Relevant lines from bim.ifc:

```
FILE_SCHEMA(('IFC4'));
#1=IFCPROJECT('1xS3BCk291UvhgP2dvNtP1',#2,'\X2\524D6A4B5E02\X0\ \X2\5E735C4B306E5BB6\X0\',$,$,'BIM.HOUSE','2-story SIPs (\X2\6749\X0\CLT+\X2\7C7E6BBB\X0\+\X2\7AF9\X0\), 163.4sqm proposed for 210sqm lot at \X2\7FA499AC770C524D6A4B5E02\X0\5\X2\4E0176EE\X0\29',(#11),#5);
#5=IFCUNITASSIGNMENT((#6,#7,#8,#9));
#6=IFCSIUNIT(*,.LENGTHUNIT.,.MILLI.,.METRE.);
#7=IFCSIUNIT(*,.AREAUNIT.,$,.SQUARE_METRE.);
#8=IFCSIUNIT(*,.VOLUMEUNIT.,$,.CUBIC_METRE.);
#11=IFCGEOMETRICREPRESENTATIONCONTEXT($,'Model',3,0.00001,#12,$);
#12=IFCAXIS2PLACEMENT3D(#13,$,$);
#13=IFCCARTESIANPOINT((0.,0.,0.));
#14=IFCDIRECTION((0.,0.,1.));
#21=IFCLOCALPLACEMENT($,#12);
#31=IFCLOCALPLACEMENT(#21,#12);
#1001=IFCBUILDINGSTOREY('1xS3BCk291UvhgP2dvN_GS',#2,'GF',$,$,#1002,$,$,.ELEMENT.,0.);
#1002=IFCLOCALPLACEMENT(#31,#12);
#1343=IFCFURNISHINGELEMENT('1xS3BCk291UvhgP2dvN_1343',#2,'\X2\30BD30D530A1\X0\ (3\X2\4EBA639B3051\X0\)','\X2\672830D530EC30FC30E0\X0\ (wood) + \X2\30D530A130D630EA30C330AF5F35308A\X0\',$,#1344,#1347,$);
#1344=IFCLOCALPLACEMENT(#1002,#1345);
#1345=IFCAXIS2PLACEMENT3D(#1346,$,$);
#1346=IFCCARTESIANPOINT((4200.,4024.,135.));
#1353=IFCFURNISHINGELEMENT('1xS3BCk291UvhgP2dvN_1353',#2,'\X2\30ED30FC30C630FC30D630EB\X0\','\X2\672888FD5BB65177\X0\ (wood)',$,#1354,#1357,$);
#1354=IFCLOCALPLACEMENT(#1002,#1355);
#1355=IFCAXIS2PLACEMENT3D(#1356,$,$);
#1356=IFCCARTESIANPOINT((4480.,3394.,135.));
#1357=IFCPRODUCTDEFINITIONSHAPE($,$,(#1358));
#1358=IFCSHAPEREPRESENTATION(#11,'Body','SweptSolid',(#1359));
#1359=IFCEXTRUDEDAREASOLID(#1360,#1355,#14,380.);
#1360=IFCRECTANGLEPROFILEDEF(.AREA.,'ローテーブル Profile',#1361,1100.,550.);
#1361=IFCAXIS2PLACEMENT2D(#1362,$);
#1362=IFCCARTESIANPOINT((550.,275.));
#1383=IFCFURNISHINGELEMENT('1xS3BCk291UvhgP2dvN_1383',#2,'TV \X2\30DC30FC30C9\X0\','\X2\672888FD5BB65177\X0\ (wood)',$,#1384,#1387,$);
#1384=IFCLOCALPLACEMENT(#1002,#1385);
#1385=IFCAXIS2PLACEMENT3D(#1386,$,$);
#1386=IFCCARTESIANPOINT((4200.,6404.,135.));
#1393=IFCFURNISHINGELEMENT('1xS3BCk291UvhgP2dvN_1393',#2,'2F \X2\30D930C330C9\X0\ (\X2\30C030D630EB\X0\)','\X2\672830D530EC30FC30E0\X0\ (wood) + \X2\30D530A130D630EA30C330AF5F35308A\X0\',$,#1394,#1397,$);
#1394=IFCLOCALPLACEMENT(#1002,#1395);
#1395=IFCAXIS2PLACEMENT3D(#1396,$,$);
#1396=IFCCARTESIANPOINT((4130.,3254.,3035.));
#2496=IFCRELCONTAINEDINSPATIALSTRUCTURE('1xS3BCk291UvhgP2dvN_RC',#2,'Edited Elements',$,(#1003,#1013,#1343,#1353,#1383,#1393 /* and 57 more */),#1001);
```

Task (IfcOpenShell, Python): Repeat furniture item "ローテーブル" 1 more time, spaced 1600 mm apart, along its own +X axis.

```python
import ifcopenshell
import ifcopenshell.api.geometry
import ifcopenshell.api.root
import ifcopenshell.util.element
import ifcopenshell.util.placement

model = ifcopenshell.open("bim.ifc")


def reuse_history(source, copy):
    """copy_class also copies each property set's owner history, people and application; keep the originals."""
    for rel in copy.IsDefinedBy:
        if rel.is_a("IfcRelDefinesByProperties") and (history := rel.RelatingPropertyDefinition.OwnerHistory):
            rel.RelatingPropertyDefinition.OwnerHistory = source.OwnerHistory
            ifcopenshell.util.element.remove_deep2(model, history)


source = model.by_guid("1xS3BCk291UvhgP2dvN_1353")
base = ifcopenshell.util.placement.get_local_placement(source.ObjectPlacement)
step = base[:3, 0] * 1600.0

for i in range(1, 2):
    copy = ifcopenshell.api.root.copy_class(model, product=source)
    copy.Representation = ifcopenshell.util.element.copy_deep(
        model, source.Representation, exclude=["IfcGeometricRepresentationContext", "IfcRepresentationMap"]
    )
    reuse_history(source, copy)
    matrix = base.copy()
    matrix[:3, 3] += i * step
    print("added at", matrix[:3, 3].round(3) + 0.0)
    ifcopenshell.api.geometry.edit_object_placement(model, product=copy, matrix=matrix, is_si=False)

model.write("bim-out.ifc")
```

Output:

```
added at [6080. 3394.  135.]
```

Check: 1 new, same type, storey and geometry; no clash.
